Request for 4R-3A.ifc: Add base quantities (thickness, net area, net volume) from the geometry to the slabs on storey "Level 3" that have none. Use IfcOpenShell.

First a look at what the model holds.

```python
import ifcopenshell
import ifcopenshell.util.element
import ifcopenshell.util.unit

model = ifcopenshell.open("4R-3A.ifc")
print(model.schema)
for unit_type in ("LENGTHUNIT", "AREAUNIT", "VOLUMEUNIT"):
    print(unit_type, ifcopenshell.util.unit.calculate_unit_scale(model, unit_type))
storey = next(s for s in model.by_type("IfcBuildingStorey") if s.Name == "Level 3")
slabs = [e for e in ifcopenshell.util.element.get_decomposition(storey) if e.is_a("IfcSlab")]
for e in sorted(slabs, key=lambda e: e.id()):
    print(e.id(), e.is_a(), e.Name, list(ifcopenshell.util.element.get_psets(e, qtos_only=True)), sep=" | ")
```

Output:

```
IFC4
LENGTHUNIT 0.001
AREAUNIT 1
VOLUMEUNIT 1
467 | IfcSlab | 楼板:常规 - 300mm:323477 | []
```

```python
import ifcopenshell
import ifcopenshell.api.pset
import ifcopenshell.geom
import ifcopenshell.util.element
import ifcopenshell.util.shape
import ifcopenshell.util.unit

model = ifcopenshell.open("4R-3A.ifc")
unit_scale = ifcopenshell.util.unit.calculate_unit_scale(model)
area_scale = ifcopenshell.util.unit.calculate_unit_scale(model, "AREAUNIT")
volume_scale = ifcopenshell.util.unit.calculate_unit_scale(model, "VOLUMEUNIT")
settings = ifcopenshell.geom.settings()

storey = next(s for s in model.by_type("IfcBuildingStorey") if s.Name == "Level 3")
slabs = [e for e in ifcopenshell.util.element.get_decomposition(storey) if e.is_a("IfcSlab")]

for e in sorted(slabs, key=lambda e: e.id()):
    if ifcopenshell.util.element.get_psets(e, qtos_only=True, should_inherit=False):
        continue
    # Geometry comes back in metres, in the element's own axes.
    shape = ifcopenshell.geom.create_shape(settings, e)
    values = {
        "Width": ifcopenshell.util.shape.get_z(shape.geometry) / unit_scale,
        "NetArea": ifcopenshell.util.shape.get_footprint_area(shape.geometry) / area_scale,
        "NetVolume": ifcopenshell.util.shape.get_volume(shape.geometry) / volume_scale,
    }
    qto = ifcopenshell.api.pset.add_qto(model, product=e, name="Qto_SlabBaseQuantities")
    ifcopenshell.api.pset.edit_qto(model, qto=qto, properties=values)
    print(e.id(), {k: round(v, 3) for k, v in values.items()})

model.write("4R-3A_rev.ifc")
```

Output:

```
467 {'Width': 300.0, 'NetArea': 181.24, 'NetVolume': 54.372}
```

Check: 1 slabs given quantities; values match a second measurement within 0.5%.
